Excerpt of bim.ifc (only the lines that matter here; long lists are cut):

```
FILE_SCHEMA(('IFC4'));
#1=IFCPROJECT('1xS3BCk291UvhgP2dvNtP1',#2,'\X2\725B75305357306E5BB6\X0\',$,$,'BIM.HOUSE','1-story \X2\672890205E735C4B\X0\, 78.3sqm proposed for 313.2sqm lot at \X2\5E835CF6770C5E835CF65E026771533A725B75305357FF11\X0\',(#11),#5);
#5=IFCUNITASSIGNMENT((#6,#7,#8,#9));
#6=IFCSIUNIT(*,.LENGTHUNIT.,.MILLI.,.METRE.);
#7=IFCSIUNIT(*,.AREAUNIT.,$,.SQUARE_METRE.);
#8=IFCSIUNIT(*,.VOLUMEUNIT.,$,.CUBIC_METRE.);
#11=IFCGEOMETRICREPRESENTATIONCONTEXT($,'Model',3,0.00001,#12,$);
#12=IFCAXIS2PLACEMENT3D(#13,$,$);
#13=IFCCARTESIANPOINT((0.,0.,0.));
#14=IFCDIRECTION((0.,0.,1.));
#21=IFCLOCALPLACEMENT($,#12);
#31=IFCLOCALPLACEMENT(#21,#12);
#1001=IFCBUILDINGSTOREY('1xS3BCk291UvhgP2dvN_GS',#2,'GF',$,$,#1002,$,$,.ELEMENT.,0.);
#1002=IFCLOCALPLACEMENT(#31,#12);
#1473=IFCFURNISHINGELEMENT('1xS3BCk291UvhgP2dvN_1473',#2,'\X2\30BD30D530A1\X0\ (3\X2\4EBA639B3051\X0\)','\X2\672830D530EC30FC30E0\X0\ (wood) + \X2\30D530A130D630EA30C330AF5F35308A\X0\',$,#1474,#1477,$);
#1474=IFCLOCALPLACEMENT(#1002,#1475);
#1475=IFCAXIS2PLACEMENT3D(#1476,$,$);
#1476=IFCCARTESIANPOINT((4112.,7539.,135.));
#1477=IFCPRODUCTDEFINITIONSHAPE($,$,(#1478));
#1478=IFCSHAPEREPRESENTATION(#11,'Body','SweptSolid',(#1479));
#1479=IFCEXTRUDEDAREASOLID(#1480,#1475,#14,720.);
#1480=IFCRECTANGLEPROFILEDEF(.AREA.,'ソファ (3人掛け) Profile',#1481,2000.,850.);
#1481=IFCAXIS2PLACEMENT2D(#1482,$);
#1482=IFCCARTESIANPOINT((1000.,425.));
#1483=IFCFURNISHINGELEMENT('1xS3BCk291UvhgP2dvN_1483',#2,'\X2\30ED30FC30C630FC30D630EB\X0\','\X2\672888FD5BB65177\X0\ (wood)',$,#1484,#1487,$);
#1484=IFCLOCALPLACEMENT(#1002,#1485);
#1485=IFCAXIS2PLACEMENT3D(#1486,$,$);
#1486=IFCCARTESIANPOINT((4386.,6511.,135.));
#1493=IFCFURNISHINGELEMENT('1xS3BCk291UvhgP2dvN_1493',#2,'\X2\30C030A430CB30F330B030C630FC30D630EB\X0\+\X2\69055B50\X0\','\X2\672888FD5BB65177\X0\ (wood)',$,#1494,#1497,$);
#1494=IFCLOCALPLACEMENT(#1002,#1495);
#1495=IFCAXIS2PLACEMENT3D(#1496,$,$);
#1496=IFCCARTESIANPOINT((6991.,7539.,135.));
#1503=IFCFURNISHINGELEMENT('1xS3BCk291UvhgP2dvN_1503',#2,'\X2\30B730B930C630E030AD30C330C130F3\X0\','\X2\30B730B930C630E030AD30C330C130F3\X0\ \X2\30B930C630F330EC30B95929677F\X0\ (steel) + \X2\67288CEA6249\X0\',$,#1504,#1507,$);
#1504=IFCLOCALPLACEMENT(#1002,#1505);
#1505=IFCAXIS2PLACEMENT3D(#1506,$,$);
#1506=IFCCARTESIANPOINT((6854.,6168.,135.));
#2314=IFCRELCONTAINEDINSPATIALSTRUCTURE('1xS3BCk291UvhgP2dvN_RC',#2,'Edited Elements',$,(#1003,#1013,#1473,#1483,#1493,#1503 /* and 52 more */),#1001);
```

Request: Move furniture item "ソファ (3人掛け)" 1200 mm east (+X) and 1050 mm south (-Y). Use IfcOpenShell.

```python
import ifcopenshell
import ifcopenshell.api.geometry
import ifcopenshell.util.placement

model = ifcopenshell.open("bim.ifc")

item = model.by_guid("1xS3BCk291UvhgP2dvN_1473")
matrix = ifcopenshell.util.placement.get_local_placement(item.ObjectPlacement)
matrix[0, 3] += 1200.0
matrix[1, 3] -= 1050.0
ifcopenshell.api.geometry.edit_object_placement(model, product=item, matrix=matrix, is_si=False)

print(ifcopenshell.util.placement.get_local_placement(item.ObjectPlacement).round(3) + 0.0)

model.write("bim_v2.ifc")
```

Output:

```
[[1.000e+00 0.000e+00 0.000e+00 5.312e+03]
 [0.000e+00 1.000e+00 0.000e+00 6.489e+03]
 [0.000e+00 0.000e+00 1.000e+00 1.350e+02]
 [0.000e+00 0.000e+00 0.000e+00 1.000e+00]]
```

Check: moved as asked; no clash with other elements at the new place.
